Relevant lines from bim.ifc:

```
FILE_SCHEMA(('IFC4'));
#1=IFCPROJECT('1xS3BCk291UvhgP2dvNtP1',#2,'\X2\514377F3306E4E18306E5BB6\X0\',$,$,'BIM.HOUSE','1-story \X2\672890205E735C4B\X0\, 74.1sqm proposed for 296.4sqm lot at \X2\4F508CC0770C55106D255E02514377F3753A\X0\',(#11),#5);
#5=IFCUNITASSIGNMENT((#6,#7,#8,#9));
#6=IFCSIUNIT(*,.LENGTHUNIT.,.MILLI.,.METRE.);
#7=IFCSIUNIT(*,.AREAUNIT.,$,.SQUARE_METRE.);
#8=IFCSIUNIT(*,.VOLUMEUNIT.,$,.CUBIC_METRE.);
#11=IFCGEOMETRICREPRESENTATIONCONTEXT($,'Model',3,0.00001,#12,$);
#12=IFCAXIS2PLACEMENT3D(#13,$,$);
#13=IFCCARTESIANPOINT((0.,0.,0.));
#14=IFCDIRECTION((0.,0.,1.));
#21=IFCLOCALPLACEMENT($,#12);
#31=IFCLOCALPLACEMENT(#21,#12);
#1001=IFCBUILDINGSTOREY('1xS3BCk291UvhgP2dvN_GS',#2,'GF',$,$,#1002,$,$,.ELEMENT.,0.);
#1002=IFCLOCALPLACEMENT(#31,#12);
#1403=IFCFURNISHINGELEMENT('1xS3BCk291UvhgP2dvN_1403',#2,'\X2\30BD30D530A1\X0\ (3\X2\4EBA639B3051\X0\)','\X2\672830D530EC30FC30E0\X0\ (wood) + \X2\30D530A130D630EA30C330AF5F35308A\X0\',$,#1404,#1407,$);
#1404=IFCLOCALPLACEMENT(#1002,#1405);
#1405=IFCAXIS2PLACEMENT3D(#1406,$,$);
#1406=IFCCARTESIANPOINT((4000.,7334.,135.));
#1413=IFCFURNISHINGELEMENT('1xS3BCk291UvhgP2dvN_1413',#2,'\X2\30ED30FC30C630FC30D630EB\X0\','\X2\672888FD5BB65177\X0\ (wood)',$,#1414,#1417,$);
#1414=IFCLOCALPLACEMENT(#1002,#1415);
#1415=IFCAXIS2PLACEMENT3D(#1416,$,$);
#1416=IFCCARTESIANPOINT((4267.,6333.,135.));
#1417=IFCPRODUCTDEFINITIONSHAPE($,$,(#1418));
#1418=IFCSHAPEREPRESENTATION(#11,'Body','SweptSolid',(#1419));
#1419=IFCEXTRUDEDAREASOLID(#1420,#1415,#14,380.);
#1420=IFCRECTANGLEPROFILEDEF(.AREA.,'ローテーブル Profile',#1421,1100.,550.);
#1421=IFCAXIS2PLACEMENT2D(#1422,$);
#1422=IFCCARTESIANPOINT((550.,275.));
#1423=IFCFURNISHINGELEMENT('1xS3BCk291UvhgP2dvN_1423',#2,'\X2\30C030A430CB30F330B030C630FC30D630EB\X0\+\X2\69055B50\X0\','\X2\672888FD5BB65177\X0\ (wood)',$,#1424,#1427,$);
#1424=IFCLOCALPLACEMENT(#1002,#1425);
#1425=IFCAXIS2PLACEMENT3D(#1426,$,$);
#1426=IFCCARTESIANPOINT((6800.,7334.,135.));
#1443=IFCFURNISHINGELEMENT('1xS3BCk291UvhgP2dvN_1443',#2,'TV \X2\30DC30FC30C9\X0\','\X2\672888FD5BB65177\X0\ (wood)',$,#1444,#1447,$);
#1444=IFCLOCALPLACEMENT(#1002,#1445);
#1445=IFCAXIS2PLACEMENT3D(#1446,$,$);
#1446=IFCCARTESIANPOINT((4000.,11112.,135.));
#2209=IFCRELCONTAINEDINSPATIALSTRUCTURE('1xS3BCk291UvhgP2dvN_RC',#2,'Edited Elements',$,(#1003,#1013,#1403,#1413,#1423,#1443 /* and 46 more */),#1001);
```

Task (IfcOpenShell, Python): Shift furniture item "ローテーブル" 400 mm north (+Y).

```python
import ifcopenshell
import ifcopenshell.api.geometry
import ifcopenshell.util.placement
import ifcopenshell.util.unit

model = ifcopenshell.open("bim.ifc")
unit_scale = ifcopenshell.util.unit.calculate_unit_scale(model)

item = model.by_id(1413)
matrix = ifcopenshell.util.placement.get_local_placement(item.ObjectPlacement)
matrix[1, 3] += 0.4 / unit_scale
ifcopenshell.api.geometry.edit_object_placement(model, product=item, matrix=matrix, is_si=False)

print(ifcopenshell.util.placement.get_local_placement(item.ObjectPlacement).round(3) + 0.0)

model.write("bim_rev.ifc")
```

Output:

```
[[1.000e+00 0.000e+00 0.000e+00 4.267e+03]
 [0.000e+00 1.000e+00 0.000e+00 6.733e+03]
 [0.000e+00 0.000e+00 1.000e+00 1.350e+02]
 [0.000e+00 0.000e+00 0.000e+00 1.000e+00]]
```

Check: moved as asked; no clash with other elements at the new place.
